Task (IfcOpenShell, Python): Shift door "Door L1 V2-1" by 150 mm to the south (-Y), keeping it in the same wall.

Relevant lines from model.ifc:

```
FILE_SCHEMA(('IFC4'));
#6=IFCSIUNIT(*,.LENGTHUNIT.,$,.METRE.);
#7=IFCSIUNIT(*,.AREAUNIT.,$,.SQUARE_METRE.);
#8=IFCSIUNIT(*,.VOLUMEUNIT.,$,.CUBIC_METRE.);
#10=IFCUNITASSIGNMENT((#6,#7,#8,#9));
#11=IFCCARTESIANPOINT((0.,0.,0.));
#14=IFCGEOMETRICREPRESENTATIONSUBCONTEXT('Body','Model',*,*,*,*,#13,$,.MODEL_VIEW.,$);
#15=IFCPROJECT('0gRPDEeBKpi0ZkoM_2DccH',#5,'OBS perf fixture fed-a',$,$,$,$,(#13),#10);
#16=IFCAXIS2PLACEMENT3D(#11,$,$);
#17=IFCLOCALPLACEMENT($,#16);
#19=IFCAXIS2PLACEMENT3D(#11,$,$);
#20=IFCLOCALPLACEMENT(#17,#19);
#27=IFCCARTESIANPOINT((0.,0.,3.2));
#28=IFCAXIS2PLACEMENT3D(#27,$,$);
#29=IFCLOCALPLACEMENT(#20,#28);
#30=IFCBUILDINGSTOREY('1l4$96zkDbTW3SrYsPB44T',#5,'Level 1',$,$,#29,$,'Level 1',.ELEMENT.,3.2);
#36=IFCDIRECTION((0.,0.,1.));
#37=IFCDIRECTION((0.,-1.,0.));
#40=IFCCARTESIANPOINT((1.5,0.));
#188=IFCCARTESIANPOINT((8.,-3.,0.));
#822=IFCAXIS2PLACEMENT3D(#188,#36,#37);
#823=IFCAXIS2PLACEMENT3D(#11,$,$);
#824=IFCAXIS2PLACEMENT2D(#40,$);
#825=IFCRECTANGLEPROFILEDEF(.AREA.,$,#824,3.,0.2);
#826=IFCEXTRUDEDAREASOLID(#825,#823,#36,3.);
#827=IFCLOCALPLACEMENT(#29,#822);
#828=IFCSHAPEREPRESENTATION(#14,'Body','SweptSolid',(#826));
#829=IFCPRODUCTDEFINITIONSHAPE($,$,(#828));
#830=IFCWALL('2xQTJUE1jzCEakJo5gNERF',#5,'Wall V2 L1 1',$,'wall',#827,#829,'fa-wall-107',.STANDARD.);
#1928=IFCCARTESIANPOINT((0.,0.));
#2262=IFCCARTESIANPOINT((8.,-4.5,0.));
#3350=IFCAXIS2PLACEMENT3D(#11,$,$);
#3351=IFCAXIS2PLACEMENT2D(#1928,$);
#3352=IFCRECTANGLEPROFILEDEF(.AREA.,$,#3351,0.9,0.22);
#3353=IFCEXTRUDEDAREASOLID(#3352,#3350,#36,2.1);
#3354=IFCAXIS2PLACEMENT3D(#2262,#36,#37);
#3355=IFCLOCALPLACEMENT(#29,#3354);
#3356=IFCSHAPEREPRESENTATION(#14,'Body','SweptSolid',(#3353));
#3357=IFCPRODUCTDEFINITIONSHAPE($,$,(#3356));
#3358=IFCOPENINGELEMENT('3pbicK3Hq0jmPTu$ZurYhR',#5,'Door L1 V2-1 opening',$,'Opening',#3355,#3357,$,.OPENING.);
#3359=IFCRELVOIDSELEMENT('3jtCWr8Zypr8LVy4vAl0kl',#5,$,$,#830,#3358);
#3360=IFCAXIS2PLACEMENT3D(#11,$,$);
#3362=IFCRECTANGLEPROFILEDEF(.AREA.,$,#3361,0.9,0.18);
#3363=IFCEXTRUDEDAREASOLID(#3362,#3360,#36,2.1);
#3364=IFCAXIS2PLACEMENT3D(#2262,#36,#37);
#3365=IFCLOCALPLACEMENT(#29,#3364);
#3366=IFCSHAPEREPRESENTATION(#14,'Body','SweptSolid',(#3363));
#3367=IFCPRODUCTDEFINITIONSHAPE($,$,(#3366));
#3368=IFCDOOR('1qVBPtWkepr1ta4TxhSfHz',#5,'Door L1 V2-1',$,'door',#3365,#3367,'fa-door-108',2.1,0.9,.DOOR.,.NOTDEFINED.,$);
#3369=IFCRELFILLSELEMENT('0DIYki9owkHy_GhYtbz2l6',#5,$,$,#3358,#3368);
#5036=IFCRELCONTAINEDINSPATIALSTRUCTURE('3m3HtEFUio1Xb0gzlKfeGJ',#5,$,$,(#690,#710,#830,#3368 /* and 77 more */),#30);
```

```python
import ifcopenshell
import ifcopenshell.api.geometry
import ifcopenshell.util.placement
import ifcopenshell.util.unit

model = ifcopenshell.open("model.ifc")
unit_scale = ifcopenshell.util.unit.calculate_unit_scale(model)

door = model.by_id(3368)
opening = door.FillsVoids[0].RelatingOpeningElement
wall = opening.VoidsElements[0].RelatingBuildingElement

wall_matrix = ifcopenshell.util.placement.get_local_placement(wall.ObjectPlacement)
shift = wall_matrix[:3, 0] * 0.15 / unit_scale
before = ifcopenshell.util.placement.get_local_placement(door.ObjectPlacement)[:3, 3].copy()

# The door is not placed relative to its opening, so move both.
for product in (opening, door):
    matrix = ifcopenshell.util.placement.get_local_placement(product.ObjectPlacement)
    matrix[:3, 3] += shift
    ifcopenshell.api.geometry.edit_object_placement(model, product=product, matrix=matrix, is_si=False)

after = ifcopenshell.util.placement.get_local_placement(door.ObjectPlacement)[:3, 3]
print("door moved by", (after - before).round(3) + 0.0)

model.write("model_edited.ifc")
```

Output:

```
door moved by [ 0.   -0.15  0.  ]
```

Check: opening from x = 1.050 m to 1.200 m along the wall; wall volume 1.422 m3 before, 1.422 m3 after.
